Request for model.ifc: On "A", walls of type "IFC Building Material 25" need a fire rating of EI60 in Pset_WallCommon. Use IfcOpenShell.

First a look at what the model holds.

```python
import ifcopenshell
import ifcopenshell.util.element

model = ifcopenshell.open("model.ifc")
print(model.schema)
storey = next(s for s in model.by_type("IfcBuildingStorey") if s.Name == "A")
walls = [e for e in ifcopenshell.util.element.get_decomposition(storey) if e.is_a("IfcWall")]
seen = {}
for e in walls:
    element_type = ifcopenshell.util.element.get_type(e)
    key = (element_type.Name if element_type != e and element_type else None, ifcopenshell.util.element.get_pset(e, "Pset_WallCommon", "FireRating"))
    seen[key] = seen.get(key, 0) + 1
for (name, value), count in sorted(seen.items(), key=str):
    print(count, "x", name, "|", value)
```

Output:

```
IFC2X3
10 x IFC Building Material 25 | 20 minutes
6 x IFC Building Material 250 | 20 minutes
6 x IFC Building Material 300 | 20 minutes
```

```python
import ifcopenshell
import ifcopenshell.api.pset
import ifcopenshell.util.element

model = ifcopenshell.open("model.ifc")

storey = next(s for s in model.by_type("IfcBuildingStorey") if s.Name == "A")
walls = [e for e in ifcopenshell.util.element.get_decomposition(storey) if e.is_a("IfcWall")]

count = 0
for e in walls:
    element_type = ifcopenshell.util.element.get_type(e)
    if element_type in (None, e) or element_type.Name != "IFC Building Material 25":
        continue
    # add_pset returns the element's existing set when there is one.
    pset = ifcopenshell.api.pset.add_pset(model, product=e, name="Pset_WallCommon")
    ifcopenshell.api.pset.edit_pset(model, pset=pset, properties={"FireRating": "EI60"})
    count += 1

print(count, "walls updated")

model.write("model-out.ifc")
```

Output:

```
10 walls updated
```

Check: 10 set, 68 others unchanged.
